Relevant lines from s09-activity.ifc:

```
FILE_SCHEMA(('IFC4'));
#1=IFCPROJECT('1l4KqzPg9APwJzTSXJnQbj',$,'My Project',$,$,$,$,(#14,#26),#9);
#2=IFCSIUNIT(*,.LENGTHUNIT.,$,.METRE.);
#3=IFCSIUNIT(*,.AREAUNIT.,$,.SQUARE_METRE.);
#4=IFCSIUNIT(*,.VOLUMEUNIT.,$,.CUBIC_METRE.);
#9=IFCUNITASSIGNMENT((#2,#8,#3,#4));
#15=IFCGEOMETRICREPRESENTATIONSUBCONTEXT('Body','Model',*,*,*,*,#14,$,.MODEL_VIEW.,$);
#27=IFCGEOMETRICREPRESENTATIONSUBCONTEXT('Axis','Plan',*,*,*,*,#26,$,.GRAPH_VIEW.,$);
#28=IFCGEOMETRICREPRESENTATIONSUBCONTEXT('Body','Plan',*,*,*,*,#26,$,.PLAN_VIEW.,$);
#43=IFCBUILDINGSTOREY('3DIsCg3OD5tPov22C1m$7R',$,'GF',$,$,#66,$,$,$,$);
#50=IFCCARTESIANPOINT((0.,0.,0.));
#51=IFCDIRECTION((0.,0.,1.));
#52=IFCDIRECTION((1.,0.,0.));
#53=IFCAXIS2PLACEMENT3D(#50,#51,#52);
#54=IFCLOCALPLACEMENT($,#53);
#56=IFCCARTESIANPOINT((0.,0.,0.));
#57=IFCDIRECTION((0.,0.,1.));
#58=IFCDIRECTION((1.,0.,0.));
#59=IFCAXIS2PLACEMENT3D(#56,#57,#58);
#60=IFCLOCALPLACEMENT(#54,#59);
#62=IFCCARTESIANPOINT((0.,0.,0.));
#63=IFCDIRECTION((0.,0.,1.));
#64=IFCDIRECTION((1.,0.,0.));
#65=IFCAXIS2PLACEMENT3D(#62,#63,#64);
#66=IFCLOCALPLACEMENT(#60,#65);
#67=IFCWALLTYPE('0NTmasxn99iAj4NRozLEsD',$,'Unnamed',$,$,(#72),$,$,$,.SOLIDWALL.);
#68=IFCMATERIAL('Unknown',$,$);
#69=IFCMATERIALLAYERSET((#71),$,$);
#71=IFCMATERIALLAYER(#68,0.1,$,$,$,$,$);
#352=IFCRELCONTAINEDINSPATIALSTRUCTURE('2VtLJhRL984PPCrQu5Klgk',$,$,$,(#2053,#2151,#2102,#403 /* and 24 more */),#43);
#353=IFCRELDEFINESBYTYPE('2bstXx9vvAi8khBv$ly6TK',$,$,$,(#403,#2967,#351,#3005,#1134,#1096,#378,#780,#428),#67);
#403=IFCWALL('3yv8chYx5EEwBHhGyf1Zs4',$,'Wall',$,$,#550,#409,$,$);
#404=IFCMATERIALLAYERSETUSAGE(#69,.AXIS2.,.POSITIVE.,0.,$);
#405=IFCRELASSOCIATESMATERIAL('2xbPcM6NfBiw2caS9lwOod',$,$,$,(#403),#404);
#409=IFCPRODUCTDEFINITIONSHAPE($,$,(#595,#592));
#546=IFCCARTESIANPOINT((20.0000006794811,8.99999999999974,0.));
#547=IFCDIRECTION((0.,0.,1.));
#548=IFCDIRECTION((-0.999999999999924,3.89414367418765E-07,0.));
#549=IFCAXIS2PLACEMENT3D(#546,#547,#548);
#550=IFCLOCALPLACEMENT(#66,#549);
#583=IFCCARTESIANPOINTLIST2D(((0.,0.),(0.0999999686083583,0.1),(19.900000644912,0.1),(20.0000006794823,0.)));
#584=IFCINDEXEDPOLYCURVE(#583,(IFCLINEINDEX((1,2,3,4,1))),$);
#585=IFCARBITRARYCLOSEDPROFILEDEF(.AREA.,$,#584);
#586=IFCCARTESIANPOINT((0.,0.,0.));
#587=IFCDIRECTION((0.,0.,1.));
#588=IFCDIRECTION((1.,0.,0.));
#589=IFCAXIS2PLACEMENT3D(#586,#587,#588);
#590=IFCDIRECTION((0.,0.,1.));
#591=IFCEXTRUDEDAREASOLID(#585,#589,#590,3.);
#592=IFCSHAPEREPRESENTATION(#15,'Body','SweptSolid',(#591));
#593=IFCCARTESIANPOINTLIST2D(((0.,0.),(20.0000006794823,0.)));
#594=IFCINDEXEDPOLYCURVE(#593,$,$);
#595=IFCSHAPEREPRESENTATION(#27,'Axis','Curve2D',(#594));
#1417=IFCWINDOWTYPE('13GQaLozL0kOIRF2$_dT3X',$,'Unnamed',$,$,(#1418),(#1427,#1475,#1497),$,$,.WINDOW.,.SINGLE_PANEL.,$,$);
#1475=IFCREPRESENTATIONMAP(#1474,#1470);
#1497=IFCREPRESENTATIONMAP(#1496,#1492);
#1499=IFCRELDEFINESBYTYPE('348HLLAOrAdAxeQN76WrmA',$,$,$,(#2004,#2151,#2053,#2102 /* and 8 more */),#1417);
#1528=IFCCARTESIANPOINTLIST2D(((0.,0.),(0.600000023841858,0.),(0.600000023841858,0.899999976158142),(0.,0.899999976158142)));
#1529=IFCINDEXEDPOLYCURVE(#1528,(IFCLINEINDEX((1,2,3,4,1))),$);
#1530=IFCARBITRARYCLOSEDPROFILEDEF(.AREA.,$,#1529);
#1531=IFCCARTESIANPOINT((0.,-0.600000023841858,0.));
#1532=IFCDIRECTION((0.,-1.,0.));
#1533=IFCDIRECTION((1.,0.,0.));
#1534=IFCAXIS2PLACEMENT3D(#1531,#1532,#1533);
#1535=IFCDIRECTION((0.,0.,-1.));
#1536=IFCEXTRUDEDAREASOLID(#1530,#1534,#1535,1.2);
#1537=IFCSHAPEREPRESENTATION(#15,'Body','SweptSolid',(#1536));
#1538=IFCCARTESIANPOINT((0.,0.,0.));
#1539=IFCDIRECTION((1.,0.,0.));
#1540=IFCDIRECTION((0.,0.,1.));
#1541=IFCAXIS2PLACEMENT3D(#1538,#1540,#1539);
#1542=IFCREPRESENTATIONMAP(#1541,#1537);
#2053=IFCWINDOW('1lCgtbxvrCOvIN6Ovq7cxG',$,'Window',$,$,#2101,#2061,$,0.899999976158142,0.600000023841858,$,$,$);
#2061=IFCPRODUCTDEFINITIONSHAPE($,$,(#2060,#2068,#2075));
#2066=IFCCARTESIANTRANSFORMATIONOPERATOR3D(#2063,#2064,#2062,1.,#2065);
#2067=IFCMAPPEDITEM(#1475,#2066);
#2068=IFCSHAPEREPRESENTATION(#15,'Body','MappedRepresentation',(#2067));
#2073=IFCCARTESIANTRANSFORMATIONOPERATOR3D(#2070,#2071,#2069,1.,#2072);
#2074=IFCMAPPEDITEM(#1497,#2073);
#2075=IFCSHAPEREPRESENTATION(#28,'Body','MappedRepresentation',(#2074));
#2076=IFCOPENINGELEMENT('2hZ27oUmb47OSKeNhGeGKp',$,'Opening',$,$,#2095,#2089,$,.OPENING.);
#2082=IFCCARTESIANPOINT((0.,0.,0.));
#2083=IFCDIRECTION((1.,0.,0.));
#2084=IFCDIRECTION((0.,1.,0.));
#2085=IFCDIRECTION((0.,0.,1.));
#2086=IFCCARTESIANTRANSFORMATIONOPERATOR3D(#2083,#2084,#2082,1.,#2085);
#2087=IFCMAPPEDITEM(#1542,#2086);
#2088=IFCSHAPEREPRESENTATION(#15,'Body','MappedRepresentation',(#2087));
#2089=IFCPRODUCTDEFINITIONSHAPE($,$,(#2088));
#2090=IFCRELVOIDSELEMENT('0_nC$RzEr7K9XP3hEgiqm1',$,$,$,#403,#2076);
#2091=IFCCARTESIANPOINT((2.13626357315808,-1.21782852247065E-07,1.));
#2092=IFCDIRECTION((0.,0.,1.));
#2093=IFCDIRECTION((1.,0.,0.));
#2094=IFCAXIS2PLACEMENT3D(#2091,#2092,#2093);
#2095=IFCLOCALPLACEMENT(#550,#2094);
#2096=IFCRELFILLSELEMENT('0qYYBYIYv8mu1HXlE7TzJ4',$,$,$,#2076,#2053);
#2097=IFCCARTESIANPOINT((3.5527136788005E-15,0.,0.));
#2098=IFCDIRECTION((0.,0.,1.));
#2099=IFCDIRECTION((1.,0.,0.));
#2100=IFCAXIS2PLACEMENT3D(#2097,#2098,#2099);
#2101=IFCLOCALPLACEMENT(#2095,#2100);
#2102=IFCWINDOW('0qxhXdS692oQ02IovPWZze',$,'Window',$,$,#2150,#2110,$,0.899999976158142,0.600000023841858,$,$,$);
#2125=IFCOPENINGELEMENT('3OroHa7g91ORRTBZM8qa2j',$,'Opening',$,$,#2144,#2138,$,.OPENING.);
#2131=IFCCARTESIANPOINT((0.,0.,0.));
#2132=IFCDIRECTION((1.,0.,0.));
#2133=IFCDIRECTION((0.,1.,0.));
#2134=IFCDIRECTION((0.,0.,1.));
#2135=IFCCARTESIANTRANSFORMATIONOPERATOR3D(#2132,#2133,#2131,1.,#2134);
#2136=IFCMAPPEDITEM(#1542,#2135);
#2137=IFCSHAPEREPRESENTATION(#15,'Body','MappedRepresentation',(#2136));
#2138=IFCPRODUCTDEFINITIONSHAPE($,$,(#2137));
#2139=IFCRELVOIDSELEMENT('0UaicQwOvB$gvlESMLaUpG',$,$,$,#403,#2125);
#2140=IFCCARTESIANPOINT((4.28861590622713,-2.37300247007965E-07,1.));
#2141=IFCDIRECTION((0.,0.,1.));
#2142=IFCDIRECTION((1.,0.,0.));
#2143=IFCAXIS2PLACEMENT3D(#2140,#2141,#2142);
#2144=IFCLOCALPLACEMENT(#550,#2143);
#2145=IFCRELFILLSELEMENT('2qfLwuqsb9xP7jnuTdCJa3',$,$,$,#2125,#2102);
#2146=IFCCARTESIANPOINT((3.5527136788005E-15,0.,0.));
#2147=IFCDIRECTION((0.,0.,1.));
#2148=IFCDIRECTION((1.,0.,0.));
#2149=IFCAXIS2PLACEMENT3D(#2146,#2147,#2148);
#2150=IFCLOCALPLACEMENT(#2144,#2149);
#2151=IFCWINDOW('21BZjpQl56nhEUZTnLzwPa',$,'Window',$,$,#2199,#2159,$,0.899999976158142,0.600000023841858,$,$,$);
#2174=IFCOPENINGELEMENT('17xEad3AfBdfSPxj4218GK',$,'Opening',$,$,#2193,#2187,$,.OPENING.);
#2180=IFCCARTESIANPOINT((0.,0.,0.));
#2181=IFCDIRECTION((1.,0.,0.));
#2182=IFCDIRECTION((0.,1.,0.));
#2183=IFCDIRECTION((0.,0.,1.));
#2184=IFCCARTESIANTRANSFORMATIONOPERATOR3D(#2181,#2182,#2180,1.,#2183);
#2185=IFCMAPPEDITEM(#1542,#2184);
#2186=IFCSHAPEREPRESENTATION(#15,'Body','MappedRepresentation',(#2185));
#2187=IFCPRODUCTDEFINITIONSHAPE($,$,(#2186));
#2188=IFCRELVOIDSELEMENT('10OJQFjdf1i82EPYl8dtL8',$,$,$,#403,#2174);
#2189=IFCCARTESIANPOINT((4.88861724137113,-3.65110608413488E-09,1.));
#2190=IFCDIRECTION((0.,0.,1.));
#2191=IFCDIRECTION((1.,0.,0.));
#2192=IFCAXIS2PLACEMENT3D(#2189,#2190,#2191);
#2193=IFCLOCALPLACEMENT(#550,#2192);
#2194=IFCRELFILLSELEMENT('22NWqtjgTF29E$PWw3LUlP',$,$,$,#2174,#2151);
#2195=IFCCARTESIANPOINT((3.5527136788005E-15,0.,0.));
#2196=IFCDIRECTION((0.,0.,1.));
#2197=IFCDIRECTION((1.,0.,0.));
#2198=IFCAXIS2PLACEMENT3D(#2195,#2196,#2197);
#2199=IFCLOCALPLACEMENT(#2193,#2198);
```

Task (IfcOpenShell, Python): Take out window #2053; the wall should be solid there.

```python
import ifcopenshell
import ifcopenshell.api.feature
import ifcopenshell.api.root
import ifcopenshell.geom
import ifcopenshell.util.shape

model = ifcopenshell.open("s09-activity.ifc")
settings = ifcopenshell.geom.settings()


def volume(element):
    """Net volume in cubic metres, openings subtracted."""
    shape = ifcopenshell.geom.create_shape(settings, element)
    return ifcopenshell.util.shape.get_volume(shape.geometry)


window = model.by_guid("1lCgtbxvrCOvIN6Ovq7cxG")
opening = window.FillsVoids[0].RelatingOpeningElement
wall = opening.VoidsElements[0].RelatingBuildingElement
before = volume(wall)

ifcopenshell.api.root.remove_product(model, product=window)
ifcopenshell.api.feature.remove_feature(model, feature=opening)

after = volume(wall)

print(f"wall volume {before:.3f} -> {after:.3f} m3")

model.write("s09-activity_rev.ifc")
```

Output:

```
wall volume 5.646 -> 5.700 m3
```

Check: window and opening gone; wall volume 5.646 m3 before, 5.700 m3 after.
